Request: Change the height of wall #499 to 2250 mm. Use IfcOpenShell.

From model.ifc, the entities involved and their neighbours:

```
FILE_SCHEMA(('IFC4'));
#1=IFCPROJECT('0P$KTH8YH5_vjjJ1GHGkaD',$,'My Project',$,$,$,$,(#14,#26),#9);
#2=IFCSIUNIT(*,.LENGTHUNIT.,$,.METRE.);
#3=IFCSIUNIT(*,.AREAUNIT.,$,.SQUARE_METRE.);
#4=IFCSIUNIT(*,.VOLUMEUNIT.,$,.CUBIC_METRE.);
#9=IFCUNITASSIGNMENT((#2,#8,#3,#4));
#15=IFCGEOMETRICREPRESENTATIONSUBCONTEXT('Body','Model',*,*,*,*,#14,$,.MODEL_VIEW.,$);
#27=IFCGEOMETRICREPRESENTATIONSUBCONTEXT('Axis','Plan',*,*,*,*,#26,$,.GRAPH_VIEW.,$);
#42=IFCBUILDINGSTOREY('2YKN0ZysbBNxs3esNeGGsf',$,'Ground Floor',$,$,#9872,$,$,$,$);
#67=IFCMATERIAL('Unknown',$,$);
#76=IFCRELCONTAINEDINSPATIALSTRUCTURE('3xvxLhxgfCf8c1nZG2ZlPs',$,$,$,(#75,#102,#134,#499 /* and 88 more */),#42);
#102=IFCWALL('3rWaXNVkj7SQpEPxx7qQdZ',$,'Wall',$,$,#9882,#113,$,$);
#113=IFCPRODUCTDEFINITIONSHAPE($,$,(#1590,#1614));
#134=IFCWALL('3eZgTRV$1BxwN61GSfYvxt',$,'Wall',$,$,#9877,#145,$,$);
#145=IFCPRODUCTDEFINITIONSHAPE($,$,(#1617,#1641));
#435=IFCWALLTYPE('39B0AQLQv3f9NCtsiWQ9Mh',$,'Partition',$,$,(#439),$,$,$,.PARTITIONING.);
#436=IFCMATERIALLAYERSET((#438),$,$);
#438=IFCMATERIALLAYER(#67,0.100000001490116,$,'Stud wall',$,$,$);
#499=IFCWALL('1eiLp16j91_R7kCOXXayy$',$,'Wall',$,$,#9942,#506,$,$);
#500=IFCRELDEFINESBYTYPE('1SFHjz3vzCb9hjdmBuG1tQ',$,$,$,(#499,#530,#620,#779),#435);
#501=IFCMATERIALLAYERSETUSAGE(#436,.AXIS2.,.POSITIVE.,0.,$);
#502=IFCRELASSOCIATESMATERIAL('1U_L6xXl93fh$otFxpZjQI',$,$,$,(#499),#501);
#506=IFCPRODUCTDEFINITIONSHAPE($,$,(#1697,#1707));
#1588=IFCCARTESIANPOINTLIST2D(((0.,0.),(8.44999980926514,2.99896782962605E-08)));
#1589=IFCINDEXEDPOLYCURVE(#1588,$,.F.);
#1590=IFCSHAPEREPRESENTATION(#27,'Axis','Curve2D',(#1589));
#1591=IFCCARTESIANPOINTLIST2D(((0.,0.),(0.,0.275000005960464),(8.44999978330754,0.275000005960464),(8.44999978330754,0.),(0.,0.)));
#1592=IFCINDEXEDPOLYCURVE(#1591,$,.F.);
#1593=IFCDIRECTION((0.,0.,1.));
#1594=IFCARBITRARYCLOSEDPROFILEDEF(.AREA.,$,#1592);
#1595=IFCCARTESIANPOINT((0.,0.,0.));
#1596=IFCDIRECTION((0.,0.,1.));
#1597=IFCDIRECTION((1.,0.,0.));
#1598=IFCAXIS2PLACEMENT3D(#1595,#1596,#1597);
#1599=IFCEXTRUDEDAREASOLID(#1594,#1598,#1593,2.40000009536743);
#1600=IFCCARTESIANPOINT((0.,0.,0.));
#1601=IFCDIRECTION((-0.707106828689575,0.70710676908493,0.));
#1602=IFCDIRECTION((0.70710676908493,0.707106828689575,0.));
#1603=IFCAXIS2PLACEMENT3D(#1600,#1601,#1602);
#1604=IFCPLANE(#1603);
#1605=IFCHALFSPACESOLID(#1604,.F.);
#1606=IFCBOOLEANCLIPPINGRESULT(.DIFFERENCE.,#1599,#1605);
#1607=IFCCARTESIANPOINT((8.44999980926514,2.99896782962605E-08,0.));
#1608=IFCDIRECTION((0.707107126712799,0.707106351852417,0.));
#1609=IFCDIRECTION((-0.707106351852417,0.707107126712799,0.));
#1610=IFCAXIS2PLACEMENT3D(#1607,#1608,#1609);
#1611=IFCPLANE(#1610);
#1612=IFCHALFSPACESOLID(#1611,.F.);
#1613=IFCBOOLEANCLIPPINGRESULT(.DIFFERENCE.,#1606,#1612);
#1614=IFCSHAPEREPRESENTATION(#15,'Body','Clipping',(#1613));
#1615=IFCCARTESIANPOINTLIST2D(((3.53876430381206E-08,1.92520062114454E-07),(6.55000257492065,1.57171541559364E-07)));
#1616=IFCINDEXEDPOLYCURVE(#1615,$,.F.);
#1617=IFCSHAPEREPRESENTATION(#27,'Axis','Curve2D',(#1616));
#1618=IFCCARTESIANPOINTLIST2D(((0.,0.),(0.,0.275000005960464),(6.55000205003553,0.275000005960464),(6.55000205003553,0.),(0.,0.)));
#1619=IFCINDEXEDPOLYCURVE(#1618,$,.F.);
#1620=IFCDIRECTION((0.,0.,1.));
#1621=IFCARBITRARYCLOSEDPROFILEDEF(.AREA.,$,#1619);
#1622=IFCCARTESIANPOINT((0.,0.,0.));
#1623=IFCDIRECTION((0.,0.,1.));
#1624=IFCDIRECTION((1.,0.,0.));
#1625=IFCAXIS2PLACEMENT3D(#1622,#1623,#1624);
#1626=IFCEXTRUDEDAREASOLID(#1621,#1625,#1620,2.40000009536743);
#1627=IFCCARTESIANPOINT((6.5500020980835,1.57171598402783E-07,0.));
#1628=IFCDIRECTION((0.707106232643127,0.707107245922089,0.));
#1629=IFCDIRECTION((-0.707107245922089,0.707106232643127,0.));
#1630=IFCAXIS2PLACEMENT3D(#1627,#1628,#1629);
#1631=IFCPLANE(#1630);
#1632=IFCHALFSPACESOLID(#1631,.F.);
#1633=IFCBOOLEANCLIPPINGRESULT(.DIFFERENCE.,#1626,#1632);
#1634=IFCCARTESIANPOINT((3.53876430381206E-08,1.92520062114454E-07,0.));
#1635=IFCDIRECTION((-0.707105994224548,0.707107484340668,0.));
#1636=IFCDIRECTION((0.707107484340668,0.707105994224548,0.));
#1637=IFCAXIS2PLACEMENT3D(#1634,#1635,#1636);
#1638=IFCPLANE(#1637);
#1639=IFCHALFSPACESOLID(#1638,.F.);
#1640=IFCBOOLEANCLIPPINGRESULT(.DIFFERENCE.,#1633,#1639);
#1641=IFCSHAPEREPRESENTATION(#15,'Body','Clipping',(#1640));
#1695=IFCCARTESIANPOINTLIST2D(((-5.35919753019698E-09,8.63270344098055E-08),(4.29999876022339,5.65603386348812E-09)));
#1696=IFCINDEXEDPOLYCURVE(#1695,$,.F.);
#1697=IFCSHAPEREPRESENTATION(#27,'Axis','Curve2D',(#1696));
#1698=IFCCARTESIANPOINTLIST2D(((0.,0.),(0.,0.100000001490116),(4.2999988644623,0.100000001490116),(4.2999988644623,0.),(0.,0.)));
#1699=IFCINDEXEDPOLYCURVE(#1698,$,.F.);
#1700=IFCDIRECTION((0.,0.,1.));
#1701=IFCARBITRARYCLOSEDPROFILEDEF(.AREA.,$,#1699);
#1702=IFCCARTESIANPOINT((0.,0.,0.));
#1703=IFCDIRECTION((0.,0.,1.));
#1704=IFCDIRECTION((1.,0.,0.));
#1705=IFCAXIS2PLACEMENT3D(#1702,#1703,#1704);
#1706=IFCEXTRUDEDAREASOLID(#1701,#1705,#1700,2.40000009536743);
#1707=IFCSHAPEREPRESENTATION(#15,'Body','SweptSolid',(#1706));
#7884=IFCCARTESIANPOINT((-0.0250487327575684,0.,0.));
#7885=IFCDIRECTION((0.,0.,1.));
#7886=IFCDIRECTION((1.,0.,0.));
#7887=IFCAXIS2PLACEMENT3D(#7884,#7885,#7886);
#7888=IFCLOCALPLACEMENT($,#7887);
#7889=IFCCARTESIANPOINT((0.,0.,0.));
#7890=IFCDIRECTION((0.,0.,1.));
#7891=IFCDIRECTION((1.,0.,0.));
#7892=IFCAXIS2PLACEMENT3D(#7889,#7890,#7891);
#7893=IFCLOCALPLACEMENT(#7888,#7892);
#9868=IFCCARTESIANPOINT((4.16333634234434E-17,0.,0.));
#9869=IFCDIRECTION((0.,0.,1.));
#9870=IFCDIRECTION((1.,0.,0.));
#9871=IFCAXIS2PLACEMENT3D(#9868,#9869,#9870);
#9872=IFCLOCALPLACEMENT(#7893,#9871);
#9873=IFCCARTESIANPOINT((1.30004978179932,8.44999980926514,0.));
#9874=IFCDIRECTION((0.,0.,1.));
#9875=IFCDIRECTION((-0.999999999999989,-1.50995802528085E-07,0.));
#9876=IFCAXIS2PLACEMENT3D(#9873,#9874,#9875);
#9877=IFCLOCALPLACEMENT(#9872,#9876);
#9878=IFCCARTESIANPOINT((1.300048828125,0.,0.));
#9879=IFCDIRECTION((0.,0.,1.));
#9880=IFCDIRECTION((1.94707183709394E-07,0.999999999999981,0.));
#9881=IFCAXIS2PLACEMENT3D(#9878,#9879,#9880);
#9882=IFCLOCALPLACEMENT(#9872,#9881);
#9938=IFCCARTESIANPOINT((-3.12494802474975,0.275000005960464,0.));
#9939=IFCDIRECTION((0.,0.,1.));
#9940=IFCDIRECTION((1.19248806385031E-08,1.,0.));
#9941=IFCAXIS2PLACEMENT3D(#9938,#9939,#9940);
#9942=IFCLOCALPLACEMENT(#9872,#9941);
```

```python
import ifcopenshell
import ifcopenshell.geom
import ifcopenshell.util.representation
import ifcopenshell.util.shape
import ifcopenshell.util.unit

model = ifcopenshell.open("model.ifc")
unit_scale = ifcopenshell.util.unit.calculate_unit_scale(model)
settings = ifcopenshell.geom.settings()


def volume(element):
    """Net volume in cubic metres, openings subtracted."""
    shape = ifcopenshell.geom.create_shape(settings, element)
    return ifcopenshell.util.shape.get_volume(shape.geometry)


wall = model.by_id(499)
before = volume(wall)

body = ifcopenshell.util.representation.get_representation(wall, "Model", "Body")
solid = body.Items[0]
old_height = solid.Depth
solid.Depth = 2.25 / unit_scale
after = volume(wall)

print(f"height {old_height:g} -> {solid.Depth:g}, volume {before:.3f} -> {after:.3f} m3")

model.write("model_edited.ifc")
```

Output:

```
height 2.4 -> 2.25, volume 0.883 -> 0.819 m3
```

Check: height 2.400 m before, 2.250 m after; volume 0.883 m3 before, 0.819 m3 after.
